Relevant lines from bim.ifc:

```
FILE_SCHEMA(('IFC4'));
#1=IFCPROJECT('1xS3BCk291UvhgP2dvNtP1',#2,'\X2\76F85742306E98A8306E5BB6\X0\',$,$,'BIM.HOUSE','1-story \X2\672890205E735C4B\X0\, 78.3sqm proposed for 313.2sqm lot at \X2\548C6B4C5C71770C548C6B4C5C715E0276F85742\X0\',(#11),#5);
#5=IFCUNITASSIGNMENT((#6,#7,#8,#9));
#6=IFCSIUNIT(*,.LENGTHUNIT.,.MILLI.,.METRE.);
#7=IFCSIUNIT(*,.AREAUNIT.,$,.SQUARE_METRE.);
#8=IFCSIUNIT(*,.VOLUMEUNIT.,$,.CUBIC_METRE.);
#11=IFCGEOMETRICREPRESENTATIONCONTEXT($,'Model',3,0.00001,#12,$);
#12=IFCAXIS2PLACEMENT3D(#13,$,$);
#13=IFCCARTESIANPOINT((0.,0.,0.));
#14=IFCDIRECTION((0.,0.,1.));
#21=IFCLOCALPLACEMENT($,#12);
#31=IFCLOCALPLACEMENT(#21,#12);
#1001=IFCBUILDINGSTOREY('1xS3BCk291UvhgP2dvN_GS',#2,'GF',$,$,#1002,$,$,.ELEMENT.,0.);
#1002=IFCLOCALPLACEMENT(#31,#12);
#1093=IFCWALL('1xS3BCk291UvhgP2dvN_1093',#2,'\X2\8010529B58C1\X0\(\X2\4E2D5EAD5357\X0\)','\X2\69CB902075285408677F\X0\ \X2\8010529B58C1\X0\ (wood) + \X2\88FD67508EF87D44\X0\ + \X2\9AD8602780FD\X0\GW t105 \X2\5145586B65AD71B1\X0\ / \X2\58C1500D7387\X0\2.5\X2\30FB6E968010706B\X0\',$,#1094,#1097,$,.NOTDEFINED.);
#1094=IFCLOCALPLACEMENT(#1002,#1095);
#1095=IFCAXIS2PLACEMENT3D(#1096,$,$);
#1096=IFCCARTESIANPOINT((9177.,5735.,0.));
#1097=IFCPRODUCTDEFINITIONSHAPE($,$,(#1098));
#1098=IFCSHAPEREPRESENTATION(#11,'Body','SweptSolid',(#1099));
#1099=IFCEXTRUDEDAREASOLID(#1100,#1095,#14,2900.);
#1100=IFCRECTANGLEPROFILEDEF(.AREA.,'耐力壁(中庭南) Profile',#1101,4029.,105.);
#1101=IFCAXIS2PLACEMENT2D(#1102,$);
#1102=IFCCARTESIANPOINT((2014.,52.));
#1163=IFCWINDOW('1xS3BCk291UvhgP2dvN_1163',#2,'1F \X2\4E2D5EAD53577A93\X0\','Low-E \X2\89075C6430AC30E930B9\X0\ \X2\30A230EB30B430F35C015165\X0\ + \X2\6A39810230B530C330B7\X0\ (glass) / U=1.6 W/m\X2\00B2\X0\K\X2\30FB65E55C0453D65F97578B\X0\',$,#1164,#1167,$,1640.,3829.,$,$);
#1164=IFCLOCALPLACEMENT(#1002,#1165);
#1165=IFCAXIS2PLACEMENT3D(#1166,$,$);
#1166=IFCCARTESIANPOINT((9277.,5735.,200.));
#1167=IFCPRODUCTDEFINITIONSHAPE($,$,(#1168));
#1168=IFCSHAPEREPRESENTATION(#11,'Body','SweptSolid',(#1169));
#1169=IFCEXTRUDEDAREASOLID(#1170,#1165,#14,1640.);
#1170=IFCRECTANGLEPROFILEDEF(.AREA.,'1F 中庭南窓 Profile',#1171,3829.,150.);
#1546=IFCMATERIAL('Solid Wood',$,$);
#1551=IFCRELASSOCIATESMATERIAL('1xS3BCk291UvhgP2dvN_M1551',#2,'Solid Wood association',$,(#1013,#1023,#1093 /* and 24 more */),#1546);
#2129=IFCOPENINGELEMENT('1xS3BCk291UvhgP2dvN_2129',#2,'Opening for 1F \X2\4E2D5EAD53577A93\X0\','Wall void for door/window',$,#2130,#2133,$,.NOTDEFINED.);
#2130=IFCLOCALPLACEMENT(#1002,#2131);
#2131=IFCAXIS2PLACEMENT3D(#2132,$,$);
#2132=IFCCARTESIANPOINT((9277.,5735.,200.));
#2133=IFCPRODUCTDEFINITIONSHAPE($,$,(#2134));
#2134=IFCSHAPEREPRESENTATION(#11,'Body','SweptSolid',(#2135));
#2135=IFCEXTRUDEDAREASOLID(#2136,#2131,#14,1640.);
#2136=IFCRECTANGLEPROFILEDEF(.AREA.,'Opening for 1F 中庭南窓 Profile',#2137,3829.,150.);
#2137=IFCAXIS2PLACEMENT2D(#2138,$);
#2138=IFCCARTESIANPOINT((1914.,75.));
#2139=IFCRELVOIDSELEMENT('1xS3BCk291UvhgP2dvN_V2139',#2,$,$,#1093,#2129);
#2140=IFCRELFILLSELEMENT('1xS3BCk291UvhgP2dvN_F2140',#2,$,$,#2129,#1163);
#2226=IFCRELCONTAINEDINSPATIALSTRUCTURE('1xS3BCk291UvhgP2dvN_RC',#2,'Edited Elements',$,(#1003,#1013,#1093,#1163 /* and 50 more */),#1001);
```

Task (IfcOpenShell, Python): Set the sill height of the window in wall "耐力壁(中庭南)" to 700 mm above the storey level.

```python
import numpy as np
import ifcopenshell
import ifcopenshell.api.geometry
import ifcopenshell.geom
import ifcopenshell.util.element
import ifcopenshell.util.placement
import ifcopenshell.util.shape
import ifcopenshell.util.unit

model = ifcopenshell.open("bim.ifc")
unit_scale = ifcopenshell.util.unit.calculate_unit_scale(model)

window = model.by_guid("1xS3BCk291UvhgP2dvN_1163")
opening = window.FillsVoids[0].RelatingOpeningElement
storey = ifcopenshell.util.element.get_container(window, ifc_class="IfcBuildingStorey")
level = ifcopenshell.util.placement.get_local_placement(storey.ObjectPlacement)[2, 3]

# The opening's origin need not be at the sill, so measure its lowest point.
shape = ifcopenshell.geom.create_shape(ifcopenshell.geom.settings(), opening)
bottom = ifcopenshell.util.shape.get_shape_bottom_elevation(shape, shape.geometry) / unit_scale
dz = level + 0.7 / unit_scale - bottom

shift = np.array([0.0, 0.0, dz])
# The window is not placed relative to its opening, so move both.
for product in (opening, window):
    matrix = ifcopenshell.util.placement.get_local_placement(product.ObjectPlacement)
    matrix[:3, 3] += shift
    ifcopenshell.api.geometry.edit_object_placement(model, product=product, matrix=matrix, is_si=False)

print(f"moved by {dz * unit_scale:+.3f} m")

model.write("bim_updated.ifc")
```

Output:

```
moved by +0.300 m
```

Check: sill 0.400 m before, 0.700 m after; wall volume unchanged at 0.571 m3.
